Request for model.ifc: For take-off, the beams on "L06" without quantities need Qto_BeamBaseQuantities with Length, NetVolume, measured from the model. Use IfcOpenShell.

First a look at what the model holds.

```python
import ifcopenshell
import ifcopenshell.util.element
import ifcopenshell.util.unit

model = ifcopenshell.open("model.ifc")
print(model.schema)
for unit_type in ("LENGTHUNIT", "AREAUNIT", "VOLUMEUNIT"):
    print(unit_type, ifcopenshell.util.unit.calculate_unit_scale(model, unit_type))
storey = next(s for s in model.by_type("IfcBuildingStorey") if s.Name == "L06")
beams = [e for e in ifcopenshell.util.element.get_decomposition(storey) if e.is_a("IfcBeam")]
for e in sorted(beams, key=lambda e: e.id()):
    print(e.id(), e.is_a(), e.Name, list(ifcopenshell.util.element.get_psets(e, qtos_only=True)), sep=" | ")
```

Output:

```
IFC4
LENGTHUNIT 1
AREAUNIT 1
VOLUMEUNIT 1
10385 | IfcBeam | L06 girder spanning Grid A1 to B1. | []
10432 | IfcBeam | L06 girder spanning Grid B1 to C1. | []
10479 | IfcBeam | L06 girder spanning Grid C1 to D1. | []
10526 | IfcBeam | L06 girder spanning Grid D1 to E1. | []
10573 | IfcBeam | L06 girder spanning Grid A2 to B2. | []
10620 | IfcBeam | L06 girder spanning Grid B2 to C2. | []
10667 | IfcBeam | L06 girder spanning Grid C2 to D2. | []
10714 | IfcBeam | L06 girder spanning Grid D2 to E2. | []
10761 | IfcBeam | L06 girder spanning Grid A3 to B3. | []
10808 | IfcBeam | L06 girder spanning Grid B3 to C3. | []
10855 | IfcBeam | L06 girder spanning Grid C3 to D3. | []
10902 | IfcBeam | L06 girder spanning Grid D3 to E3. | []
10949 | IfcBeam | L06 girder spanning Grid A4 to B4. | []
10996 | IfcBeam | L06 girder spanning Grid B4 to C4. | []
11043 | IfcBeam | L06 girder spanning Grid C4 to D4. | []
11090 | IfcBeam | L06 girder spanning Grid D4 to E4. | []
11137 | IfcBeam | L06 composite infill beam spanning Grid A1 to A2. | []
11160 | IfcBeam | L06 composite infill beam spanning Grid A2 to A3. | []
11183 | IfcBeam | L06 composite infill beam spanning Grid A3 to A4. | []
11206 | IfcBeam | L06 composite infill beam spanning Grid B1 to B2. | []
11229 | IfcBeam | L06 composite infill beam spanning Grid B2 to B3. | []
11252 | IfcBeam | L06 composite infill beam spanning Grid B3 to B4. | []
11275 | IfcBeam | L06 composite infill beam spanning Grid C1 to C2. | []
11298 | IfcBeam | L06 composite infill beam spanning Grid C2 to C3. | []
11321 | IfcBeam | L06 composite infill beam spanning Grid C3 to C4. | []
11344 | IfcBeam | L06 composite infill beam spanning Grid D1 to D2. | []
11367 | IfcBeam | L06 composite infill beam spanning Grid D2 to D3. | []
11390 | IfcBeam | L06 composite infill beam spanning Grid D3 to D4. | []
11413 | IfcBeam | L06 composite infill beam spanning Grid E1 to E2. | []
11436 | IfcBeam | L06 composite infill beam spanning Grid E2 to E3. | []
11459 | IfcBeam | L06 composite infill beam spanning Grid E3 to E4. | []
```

```python
import ifcopenshell
import ifcopenshell.api.pset
import ifcopenshell.geom
import ifcopenshell.util.element
import ifcopenshell.util.shape
import ifcopenshell.util.unit

model = ifcopenshell.open("model.ifc")
unit_scale = ifcopenshell.util.unit.calculate_unit_scale(model)
volume_scale = ifcopenshell.util.unit.calculate_unit_scale(model, "VOLUMEUNIT")
settings = ifcopenshell.geom.settings()

storey = next(s for s in model.by_type("IfcBuildingStorey") if s.Name == "L06")
beams = [e for e in ifcopenshell.util.element.get_decomposition(storey) if e.is_a("IfcBeam")]

for e in sorted(beams, key=lambda e: e.id()):
    if ifcopenshell.util.element.get_psets(e, qtos_only=True, should_inherit=False):
        continue
    # Geometry comes back in metres, in the element's own axes.
    shape = ifcopenshell.geom.create_shape(settings, e)
    values = {
        "Length": ifcopenshell.util.shape.get_max_xyz(shape.geometry) / unit_scale,
        "NetVolume": ifcopenshell.util.shape.get_volume(shape.geometry) / volume_scale,
    }
    qto = ifcopenshell.api.pset.add_qto(model, product=e, name="Qto_BeamBaseQuantities")
    ifcopenshell.api.pset.edit_qto(model, qto=qto, properties=values)
    print(e.id(), {k: round(v, 3) for k, v in values.items()})

model.write("model_v2.ifc")
```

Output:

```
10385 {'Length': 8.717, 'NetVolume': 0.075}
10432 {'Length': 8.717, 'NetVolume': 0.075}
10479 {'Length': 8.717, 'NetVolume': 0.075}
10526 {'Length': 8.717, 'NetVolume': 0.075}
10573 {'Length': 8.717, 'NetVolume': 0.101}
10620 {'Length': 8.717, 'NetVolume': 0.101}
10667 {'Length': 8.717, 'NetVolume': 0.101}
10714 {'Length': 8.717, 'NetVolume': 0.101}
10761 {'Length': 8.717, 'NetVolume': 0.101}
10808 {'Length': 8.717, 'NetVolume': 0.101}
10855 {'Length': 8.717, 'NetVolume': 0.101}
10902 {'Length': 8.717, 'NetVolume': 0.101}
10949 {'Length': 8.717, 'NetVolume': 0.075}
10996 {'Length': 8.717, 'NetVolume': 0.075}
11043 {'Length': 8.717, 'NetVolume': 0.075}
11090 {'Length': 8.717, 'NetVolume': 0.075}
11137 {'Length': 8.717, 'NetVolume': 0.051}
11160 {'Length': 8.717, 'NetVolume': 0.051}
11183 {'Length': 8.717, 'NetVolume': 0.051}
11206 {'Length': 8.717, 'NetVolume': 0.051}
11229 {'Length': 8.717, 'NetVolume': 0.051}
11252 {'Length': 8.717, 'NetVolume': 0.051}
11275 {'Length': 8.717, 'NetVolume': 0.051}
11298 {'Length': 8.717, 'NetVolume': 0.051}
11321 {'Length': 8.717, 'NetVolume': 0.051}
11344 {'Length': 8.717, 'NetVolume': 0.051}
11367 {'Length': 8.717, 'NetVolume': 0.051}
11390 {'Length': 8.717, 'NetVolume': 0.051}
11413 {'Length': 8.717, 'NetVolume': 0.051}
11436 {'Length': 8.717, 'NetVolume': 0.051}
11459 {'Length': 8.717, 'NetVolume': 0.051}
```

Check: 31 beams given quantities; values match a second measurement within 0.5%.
